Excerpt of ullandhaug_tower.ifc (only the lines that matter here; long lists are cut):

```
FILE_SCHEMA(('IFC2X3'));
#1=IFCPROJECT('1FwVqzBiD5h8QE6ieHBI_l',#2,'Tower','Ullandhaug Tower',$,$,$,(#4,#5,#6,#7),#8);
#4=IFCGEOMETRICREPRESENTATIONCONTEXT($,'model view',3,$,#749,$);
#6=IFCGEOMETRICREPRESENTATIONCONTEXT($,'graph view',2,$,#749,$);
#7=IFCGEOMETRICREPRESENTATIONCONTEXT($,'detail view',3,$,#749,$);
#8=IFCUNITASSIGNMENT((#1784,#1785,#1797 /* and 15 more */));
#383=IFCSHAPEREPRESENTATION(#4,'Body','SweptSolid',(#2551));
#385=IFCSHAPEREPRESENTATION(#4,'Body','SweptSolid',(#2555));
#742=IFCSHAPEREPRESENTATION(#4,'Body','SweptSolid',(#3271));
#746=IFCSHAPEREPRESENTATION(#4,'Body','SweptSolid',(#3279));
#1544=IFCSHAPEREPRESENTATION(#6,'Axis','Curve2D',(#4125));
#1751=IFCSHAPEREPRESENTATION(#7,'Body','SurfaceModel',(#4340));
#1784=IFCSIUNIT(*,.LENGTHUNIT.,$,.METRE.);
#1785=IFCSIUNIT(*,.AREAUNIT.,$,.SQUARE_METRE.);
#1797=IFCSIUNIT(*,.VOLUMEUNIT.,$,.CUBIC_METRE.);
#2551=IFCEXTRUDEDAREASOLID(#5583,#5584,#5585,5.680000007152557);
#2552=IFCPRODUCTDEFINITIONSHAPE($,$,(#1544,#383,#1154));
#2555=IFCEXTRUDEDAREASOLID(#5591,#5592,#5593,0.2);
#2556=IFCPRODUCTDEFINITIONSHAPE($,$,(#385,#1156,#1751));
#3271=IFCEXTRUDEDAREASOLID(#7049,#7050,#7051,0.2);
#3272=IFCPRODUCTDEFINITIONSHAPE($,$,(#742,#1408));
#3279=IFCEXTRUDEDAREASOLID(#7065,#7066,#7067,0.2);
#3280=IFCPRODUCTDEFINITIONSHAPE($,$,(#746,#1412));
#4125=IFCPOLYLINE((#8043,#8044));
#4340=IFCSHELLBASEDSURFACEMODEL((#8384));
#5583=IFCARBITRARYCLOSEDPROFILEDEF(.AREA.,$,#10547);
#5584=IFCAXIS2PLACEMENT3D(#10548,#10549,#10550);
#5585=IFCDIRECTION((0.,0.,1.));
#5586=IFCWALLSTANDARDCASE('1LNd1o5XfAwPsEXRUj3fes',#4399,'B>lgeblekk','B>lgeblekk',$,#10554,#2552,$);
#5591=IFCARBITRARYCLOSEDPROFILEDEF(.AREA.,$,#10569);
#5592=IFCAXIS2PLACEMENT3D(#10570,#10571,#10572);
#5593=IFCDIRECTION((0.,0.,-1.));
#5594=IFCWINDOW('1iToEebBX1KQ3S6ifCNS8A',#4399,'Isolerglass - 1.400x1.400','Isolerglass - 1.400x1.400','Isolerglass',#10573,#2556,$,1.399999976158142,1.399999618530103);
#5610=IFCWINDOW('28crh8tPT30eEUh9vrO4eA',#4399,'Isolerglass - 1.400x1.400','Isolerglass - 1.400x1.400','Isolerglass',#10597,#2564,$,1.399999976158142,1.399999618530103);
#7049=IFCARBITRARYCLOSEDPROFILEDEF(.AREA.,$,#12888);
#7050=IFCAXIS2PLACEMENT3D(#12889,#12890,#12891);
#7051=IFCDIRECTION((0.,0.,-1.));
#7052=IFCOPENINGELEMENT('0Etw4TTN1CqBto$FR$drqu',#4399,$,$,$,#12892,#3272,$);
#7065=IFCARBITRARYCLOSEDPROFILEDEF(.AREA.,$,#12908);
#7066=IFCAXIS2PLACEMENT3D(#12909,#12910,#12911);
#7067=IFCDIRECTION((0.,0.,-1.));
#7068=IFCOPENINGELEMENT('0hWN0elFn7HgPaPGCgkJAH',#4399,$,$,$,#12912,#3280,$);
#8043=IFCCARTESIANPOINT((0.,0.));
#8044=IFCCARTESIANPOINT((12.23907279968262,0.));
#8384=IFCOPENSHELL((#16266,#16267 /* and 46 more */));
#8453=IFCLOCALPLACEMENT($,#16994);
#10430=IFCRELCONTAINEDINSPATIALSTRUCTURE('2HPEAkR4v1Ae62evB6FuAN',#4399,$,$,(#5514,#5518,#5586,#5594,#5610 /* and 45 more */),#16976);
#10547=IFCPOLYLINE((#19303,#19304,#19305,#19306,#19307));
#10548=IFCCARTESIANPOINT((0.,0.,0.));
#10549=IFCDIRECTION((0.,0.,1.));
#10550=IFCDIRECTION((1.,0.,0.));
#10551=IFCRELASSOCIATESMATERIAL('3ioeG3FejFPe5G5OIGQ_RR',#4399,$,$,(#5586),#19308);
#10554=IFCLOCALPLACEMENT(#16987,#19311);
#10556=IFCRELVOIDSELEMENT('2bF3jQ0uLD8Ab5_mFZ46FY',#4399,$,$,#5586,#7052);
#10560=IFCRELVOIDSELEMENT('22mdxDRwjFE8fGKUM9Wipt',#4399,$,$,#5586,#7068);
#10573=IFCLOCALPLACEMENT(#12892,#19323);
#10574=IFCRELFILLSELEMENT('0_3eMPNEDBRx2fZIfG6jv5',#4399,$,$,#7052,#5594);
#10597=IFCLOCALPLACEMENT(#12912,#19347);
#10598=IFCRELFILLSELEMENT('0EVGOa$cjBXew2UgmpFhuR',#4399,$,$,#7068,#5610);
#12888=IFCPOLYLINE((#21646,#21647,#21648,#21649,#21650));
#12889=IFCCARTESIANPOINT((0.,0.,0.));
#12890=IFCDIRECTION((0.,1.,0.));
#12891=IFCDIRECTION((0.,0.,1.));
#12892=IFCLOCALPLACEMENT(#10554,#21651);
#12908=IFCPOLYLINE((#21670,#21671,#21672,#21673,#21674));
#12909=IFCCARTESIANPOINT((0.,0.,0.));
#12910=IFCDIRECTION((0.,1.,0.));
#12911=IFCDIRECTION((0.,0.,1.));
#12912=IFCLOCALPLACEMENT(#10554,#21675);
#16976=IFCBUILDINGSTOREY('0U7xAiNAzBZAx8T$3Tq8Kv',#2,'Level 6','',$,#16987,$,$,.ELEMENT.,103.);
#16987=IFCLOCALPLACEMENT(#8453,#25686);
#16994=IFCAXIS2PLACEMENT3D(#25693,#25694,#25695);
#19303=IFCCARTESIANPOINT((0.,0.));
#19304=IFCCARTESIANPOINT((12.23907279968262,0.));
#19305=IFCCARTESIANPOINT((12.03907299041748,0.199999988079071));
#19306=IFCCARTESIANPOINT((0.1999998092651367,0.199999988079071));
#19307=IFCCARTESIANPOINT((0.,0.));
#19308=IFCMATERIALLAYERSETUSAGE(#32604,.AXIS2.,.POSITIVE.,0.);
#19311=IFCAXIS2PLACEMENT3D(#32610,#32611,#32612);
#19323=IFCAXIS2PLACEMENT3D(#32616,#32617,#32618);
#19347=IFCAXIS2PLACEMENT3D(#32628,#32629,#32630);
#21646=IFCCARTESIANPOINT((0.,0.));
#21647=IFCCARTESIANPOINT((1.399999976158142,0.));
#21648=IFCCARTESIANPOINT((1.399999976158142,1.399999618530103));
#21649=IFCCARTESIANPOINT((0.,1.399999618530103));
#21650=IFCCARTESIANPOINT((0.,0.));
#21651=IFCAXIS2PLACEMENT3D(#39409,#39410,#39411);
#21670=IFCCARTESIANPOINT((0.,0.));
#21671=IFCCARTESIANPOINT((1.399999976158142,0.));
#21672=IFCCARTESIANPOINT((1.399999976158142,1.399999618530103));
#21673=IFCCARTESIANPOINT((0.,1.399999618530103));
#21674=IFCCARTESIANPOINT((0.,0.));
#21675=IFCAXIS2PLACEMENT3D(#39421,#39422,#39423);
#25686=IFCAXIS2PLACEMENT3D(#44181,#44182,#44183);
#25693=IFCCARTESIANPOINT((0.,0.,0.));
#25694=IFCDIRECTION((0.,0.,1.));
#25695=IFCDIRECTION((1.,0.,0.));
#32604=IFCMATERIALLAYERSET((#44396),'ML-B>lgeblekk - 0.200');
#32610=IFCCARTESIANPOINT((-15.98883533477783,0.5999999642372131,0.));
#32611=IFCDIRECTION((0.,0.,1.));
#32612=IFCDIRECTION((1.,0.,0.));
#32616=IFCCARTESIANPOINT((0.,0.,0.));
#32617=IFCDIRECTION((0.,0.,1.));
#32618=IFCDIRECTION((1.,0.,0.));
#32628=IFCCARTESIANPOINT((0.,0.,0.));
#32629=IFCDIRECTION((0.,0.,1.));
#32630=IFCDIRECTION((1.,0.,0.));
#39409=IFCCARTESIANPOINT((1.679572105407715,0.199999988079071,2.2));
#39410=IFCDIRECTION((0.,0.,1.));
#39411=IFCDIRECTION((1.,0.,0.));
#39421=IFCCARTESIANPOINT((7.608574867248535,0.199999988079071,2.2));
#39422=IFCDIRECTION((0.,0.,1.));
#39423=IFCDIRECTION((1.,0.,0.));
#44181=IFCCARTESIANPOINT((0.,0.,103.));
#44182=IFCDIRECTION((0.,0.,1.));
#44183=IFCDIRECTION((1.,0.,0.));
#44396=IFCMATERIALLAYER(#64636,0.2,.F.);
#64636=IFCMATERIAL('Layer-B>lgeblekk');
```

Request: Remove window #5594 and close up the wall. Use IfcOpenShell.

```python
import ifcopenshell
import ifcopenshell.api.feature
import ifcopenshell.api.root
import ifcopenshell.geom
import ifcopenshell.util.shape

model = ifcopenshell.open("ullandhaug_tower.ifc")
settings = ifcopenshell.geom.settings()


def volume(element):
    """Net volume in cubic metres, openings subtracted."""
    shape = ifcopenshell.geom.create_shape(settings, element)
    return ifcopenshell.util.shape.get_volume(shape.geometry)


window = model.by_guid("1iToEebBX1KQ3S6ifCNS8A")
opening = window.FillsVoids[0].RelatingOpeningElement
wall = opening.VoidsElements[0].RelatingBuildingElement
before = volume(wall)

ifcopenshell.api.root.remove_product(model, product=window)
ifcopenshell.api.feature.remove_feature(model, feature=opening)

after = volume(wall)

print(f"wall volume {before:.3f} -> {after:.3f} m3")

model.write("ullandhaug_tower_edited.ifc")
```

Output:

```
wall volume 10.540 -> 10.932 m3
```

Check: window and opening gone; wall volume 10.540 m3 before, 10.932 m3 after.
